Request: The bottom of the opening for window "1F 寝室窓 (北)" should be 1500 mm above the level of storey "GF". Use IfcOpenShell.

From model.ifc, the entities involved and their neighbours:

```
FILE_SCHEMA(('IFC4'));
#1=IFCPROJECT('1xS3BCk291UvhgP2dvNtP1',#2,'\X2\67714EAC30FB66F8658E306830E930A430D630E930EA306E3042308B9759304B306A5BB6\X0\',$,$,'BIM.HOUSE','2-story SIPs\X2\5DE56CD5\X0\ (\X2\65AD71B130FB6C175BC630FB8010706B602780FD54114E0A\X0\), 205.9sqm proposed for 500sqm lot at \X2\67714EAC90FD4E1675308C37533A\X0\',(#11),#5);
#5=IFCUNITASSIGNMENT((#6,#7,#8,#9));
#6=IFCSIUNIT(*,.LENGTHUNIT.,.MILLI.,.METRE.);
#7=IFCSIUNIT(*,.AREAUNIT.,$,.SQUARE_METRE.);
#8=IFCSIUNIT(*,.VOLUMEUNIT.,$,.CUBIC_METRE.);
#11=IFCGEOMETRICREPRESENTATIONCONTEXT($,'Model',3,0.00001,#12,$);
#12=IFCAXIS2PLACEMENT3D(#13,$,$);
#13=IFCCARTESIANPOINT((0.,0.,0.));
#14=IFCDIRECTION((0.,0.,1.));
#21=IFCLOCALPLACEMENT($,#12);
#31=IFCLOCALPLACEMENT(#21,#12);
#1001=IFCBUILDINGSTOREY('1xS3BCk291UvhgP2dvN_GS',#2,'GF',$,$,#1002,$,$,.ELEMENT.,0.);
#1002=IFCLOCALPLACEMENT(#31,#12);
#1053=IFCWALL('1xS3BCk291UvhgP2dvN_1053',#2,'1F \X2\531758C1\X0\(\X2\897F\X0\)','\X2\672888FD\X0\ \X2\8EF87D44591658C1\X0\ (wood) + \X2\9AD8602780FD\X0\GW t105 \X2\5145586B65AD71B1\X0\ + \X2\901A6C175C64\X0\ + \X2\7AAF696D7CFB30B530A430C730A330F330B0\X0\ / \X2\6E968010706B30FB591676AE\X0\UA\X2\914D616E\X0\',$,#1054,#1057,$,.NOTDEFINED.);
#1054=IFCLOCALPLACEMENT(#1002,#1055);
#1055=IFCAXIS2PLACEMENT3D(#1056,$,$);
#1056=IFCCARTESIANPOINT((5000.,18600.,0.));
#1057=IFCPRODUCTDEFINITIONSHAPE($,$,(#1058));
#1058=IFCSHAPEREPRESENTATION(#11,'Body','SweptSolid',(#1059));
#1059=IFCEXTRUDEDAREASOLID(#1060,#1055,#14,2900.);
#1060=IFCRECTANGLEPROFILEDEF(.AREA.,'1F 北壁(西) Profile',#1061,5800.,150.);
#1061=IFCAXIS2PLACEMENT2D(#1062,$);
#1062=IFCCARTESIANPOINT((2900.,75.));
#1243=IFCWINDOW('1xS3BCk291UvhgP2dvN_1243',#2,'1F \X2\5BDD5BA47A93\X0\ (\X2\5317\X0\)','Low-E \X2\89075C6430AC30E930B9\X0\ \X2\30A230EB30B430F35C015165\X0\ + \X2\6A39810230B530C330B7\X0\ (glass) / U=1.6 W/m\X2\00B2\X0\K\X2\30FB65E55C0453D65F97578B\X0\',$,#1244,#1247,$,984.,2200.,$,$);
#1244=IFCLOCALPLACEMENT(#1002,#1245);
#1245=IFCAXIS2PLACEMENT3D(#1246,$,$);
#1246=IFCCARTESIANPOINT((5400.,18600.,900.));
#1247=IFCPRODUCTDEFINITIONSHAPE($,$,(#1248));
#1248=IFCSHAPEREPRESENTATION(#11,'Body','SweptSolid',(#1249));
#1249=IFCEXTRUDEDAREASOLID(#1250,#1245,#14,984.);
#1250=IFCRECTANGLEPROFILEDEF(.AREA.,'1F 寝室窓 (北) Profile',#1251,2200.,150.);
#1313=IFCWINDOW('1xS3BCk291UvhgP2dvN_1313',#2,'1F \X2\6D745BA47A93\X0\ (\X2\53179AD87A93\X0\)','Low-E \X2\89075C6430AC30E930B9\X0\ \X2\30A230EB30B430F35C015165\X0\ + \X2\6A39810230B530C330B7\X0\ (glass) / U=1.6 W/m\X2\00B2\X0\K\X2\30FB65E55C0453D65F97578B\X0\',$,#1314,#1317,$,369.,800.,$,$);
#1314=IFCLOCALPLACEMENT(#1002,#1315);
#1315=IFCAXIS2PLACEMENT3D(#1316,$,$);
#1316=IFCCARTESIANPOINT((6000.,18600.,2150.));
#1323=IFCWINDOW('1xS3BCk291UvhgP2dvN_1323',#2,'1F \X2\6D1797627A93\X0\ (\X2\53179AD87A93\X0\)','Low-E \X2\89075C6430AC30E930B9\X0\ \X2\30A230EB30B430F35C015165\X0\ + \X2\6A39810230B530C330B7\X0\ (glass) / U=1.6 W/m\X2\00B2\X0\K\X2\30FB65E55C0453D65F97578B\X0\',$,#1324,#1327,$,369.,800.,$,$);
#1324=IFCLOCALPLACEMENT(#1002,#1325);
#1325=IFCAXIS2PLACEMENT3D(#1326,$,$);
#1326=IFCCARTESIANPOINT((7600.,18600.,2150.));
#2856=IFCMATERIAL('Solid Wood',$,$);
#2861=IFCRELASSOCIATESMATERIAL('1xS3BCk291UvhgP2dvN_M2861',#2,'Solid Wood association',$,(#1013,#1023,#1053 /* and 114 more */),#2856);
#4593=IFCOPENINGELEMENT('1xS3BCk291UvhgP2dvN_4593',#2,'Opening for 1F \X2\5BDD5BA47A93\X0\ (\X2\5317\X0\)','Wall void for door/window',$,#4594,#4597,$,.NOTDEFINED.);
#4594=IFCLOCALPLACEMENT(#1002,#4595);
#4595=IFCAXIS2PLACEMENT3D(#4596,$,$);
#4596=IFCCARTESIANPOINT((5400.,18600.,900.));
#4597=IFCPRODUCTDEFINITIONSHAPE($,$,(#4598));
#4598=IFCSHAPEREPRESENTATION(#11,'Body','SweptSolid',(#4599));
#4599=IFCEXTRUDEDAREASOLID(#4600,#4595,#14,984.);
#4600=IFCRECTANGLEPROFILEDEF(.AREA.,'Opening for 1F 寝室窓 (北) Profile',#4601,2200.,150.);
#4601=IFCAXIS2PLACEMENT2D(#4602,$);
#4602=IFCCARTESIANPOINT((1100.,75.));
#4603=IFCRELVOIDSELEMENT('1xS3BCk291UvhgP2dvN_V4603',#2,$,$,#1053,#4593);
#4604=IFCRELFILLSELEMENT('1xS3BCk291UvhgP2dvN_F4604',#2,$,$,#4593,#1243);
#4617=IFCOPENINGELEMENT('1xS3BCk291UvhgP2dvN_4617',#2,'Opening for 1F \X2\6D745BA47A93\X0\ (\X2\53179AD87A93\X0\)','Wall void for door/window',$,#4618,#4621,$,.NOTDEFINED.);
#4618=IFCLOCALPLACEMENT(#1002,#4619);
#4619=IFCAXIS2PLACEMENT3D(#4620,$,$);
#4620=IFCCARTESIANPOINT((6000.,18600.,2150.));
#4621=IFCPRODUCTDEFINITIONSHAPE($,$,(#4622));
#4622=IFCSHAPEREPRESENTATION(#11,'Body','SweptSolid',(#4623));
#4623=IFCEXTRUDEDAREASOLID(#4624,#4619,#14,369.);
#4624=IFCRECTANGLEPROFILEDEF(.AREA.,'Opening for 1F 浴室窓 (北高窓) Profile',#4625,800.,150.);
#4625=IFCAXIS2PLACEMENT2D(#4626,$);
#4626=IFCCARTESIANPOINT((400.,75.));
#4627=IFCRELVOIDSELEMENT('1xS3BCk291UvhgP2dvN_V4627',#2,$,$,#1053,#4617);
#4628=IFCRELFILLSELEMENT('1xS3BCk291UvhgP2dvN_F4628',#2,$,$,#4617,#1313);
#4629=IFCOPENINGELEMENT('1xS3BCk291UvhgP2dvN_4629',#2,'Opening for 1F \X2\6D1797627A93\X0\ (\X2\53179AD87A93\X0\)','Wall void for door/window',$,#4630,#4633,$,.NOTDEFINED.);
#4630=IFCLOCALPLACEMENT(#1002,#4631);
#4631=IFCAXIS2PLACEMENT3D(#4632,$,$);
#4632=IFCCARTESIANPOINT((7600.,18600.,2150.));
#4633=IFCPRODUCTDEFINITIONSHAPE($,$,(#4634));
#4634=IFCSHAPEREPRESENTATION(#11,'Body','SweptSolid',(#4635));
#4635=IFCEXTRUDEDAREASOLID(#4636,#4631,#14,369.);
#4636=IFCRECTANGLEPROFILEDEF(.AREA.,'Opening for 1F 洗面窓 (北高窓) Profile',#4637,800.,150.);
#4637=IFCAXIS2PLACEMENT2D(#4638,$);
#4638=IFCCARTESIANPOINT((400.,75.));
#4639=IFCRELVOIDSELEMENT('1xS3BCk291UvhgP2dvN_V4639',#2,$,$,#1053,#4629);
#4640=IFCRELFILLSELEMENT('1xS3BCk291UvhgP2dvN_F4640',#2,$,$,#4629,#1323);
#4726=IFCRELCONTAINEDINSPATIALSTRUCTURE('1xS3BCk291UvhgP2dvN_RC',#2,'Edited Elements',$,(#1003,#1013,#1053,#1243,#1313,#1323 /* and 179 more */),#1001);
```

```python
import numpy as np
import ifcopenshell
import ifcopenshell.api.geometry
import ifcopenshell.geom
import ifcopenshell.util.element
import ifcopenshell.util.placement
import ifcopenshell.util.shape
import ifcopenshell.util.unit

model = ifcopenshell.open("model.ifc")
unit_scale = ifcopenshell.util.unit.calculate_unit_scale(model)

window = model.by_guid("1xS3BCk291UvhgP2dvN_1243")
opening = window.FillsVoids[0].RelatingOpeningElement
storey = ifcopenshell.util.element.get_container(window, ifc_class="IfcBuildingStorey")
level = ifcopenshell.util.placement.get_local_placement(storey.ObjectPlacement)[2, 3]

# The opening's origin need not be at the sill, so measure its lowest point.
shape = ifcopenshell.geom.create_shape(ifcopenshell.geom.settings(), opening)
bottom = ifcopenshell.util.shape.get_shape_bottom_elevation(shape, shape.geometry) / unit_scale
dz = level + 1500.0 - bottom

shift = np.array([0.0, 0.0, dz])
# The window is not placed relative to its opening, so move both.
for product in (opening, window):
    matrix = ifcopenshell.util.placement.get_local_placement(product.ObjectPlacement)
    matrix[:3, 3] += shift
    ifcopenshell.api.geometry.edit_object_placement(model, product=product, matrix=matrix, is_si=False)

print(f"moved by {dz * unit_scale:+.3f} m")

model.write("model_updated.ifc")
```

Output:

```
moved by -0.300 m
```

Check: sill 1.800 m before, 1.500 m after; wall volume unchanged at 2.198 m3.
